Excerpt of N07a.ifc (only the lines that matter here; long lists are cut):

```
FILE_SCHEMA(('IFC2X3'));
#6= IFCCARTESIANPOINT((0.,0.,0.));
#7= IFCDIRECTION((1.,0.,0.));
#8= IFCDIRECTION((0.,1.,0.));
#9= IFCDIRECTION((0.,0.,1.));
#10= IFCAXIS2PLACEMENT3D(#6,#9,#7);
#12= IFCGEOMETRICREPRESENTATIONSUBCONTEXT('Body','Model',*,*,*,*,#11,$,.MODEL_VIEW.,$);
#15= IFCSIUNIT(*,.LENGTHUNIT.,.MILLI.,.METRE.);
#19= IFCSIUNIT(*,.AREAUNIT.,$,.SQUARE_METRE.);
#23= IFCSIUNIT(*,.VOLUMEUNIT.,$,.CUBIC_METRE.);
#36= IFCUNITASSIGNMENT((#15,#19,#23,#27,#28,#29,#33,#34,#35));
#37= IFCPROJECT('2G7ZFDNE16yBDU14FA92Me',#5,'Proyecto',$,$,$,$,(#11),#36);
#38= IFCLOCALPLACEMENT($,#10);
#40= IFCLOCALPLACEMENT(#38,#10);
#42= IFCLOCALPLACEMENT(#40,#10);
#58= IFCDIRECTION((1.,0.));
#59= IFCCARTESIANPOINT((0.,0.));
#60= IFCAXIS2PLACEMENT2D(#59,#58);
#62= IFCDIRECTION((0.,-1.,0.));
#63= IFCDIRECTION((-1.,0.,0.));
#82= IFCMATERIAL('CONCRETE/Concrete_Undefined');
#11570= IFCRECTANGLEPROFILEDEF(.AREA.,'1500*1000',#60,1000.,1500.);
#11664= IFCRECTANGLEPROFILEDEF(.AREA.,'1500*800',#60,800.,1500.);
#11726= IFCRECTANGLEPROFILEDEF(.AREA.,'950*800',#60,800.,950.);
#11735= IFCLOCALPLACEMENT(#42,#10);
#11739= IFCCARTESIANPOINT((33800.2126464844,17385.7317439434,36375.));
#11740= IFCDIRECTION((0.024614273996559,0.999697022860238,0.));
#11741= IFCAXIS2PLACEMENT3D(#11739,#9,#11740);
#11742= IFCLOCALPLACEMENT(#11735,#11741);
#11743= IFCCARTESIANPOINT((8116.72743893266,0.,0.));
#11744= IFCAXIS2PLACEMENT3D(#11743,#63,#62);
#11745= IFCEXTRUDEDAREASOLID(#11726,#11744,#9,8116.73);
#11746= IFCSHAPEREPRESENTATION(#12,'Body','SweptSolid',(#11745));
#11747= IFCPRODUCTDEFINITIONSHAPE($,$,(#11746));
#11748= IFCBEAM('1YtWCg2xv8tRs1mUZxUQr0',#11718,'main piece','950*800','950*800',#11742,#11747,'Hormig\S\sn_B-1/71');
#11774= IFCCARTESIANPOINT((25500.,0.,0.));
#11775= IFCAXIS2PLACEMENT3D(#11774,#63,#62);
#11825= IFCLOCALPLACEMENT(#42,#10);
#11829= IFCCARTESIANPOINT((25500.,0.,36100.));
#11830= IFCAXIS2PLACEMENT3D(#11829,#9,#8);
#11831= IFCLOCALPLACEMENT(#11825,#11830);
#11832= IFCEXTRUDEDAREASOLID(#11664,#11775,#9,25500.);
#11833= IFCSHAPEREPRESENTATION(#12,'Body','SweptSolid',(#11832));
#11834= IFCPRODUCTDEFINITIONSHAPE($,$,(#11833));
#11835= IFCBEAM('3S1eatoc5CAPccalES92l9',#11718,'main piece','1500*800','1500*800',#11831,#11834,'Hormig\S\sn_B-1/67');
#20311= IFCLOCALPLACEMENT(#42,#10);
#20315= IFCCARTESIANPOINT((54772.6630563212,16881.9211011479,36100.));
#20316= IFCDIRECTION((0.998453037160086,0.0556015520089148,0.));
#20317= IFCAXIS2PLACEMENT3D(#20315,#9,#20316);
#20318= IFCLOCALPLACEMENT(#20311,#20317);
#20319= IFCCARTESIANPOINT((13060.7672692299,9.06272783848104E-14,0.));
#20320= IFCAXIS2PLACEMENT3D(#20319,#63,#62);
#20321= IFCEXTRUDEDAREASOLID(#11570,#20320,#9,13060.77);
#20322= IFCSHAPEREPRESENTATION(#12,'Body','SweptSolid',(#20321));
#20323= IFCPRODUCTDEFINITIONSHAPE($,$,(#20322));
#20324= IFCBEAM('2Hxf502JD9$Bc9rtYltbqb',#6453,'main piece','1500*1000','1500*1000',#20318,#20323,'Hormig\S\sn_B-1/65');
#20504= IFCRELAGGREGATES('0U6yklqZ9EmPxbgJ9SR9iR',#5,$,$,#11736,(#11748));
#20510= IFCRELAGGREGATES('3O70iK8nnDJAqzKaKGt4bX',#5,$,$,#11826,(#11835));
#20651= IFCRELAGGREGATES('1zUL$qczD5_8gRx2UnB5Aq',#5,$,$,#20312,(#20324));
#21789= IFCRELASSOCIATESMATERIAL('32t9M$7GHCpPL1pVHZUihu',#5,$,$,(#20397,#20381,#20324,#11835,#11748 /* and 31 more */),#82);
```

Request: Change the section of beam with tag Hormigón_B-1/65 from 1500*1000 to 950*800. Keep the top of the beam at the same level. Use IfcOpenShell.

```python
import ifcopenshell
import ifcopenshell.util.element
import ifcopenshell.util.representation

model = ifcopenshell.open("N07a.ifc")

member = model.by_guid("2Hxf502JD9$Bc9rtYltbqb")
source = next(p for p in model.by_type("IfcRectangleProfileDef") if p.ProfileName == "950*800")

body = ifcopenshell.util.representation.get_representation(member, "Model", "Body")
solid = body.Items[0]
old_profile = solid.SweptArea

# Copy the section's sizes but keep this member's own profile position.
profile = ifcopenshell.util.element.copy(model, source)
# Profiles are centred, so shift by half the change in depth to hold the top.
shift = (old_profile.YDim - profile.YDim) / 2
x, y = old_profile.Position.Location.Coordinates
up = (0.0, 1.0)  # upwards, in the solid's own plane
location = model.createIfcCartesianPoint((x + up[0] * shift, y + up[1] * shift))
profile.Position = model.createIfcAxis2Placement2D(location, old_profile.Position.RefDirection)
solid.SweptArea = profile
if not model.get_total_inverses(old_profile):
    ifcopenshell.util.element.remove_deep2(model, old_profile)
member.Description = member.Description.replace("1500*1000", "950*800")
member.ObjectType = member.ObjectType.replace("1500*1000", "950*800")

print(solid.SweptArea)

model.write("N07a_updated.ifc")
```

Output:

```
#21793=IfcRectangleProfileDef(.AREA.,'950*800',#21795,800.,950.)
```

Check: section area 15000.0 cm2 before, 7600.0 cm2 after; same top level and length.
